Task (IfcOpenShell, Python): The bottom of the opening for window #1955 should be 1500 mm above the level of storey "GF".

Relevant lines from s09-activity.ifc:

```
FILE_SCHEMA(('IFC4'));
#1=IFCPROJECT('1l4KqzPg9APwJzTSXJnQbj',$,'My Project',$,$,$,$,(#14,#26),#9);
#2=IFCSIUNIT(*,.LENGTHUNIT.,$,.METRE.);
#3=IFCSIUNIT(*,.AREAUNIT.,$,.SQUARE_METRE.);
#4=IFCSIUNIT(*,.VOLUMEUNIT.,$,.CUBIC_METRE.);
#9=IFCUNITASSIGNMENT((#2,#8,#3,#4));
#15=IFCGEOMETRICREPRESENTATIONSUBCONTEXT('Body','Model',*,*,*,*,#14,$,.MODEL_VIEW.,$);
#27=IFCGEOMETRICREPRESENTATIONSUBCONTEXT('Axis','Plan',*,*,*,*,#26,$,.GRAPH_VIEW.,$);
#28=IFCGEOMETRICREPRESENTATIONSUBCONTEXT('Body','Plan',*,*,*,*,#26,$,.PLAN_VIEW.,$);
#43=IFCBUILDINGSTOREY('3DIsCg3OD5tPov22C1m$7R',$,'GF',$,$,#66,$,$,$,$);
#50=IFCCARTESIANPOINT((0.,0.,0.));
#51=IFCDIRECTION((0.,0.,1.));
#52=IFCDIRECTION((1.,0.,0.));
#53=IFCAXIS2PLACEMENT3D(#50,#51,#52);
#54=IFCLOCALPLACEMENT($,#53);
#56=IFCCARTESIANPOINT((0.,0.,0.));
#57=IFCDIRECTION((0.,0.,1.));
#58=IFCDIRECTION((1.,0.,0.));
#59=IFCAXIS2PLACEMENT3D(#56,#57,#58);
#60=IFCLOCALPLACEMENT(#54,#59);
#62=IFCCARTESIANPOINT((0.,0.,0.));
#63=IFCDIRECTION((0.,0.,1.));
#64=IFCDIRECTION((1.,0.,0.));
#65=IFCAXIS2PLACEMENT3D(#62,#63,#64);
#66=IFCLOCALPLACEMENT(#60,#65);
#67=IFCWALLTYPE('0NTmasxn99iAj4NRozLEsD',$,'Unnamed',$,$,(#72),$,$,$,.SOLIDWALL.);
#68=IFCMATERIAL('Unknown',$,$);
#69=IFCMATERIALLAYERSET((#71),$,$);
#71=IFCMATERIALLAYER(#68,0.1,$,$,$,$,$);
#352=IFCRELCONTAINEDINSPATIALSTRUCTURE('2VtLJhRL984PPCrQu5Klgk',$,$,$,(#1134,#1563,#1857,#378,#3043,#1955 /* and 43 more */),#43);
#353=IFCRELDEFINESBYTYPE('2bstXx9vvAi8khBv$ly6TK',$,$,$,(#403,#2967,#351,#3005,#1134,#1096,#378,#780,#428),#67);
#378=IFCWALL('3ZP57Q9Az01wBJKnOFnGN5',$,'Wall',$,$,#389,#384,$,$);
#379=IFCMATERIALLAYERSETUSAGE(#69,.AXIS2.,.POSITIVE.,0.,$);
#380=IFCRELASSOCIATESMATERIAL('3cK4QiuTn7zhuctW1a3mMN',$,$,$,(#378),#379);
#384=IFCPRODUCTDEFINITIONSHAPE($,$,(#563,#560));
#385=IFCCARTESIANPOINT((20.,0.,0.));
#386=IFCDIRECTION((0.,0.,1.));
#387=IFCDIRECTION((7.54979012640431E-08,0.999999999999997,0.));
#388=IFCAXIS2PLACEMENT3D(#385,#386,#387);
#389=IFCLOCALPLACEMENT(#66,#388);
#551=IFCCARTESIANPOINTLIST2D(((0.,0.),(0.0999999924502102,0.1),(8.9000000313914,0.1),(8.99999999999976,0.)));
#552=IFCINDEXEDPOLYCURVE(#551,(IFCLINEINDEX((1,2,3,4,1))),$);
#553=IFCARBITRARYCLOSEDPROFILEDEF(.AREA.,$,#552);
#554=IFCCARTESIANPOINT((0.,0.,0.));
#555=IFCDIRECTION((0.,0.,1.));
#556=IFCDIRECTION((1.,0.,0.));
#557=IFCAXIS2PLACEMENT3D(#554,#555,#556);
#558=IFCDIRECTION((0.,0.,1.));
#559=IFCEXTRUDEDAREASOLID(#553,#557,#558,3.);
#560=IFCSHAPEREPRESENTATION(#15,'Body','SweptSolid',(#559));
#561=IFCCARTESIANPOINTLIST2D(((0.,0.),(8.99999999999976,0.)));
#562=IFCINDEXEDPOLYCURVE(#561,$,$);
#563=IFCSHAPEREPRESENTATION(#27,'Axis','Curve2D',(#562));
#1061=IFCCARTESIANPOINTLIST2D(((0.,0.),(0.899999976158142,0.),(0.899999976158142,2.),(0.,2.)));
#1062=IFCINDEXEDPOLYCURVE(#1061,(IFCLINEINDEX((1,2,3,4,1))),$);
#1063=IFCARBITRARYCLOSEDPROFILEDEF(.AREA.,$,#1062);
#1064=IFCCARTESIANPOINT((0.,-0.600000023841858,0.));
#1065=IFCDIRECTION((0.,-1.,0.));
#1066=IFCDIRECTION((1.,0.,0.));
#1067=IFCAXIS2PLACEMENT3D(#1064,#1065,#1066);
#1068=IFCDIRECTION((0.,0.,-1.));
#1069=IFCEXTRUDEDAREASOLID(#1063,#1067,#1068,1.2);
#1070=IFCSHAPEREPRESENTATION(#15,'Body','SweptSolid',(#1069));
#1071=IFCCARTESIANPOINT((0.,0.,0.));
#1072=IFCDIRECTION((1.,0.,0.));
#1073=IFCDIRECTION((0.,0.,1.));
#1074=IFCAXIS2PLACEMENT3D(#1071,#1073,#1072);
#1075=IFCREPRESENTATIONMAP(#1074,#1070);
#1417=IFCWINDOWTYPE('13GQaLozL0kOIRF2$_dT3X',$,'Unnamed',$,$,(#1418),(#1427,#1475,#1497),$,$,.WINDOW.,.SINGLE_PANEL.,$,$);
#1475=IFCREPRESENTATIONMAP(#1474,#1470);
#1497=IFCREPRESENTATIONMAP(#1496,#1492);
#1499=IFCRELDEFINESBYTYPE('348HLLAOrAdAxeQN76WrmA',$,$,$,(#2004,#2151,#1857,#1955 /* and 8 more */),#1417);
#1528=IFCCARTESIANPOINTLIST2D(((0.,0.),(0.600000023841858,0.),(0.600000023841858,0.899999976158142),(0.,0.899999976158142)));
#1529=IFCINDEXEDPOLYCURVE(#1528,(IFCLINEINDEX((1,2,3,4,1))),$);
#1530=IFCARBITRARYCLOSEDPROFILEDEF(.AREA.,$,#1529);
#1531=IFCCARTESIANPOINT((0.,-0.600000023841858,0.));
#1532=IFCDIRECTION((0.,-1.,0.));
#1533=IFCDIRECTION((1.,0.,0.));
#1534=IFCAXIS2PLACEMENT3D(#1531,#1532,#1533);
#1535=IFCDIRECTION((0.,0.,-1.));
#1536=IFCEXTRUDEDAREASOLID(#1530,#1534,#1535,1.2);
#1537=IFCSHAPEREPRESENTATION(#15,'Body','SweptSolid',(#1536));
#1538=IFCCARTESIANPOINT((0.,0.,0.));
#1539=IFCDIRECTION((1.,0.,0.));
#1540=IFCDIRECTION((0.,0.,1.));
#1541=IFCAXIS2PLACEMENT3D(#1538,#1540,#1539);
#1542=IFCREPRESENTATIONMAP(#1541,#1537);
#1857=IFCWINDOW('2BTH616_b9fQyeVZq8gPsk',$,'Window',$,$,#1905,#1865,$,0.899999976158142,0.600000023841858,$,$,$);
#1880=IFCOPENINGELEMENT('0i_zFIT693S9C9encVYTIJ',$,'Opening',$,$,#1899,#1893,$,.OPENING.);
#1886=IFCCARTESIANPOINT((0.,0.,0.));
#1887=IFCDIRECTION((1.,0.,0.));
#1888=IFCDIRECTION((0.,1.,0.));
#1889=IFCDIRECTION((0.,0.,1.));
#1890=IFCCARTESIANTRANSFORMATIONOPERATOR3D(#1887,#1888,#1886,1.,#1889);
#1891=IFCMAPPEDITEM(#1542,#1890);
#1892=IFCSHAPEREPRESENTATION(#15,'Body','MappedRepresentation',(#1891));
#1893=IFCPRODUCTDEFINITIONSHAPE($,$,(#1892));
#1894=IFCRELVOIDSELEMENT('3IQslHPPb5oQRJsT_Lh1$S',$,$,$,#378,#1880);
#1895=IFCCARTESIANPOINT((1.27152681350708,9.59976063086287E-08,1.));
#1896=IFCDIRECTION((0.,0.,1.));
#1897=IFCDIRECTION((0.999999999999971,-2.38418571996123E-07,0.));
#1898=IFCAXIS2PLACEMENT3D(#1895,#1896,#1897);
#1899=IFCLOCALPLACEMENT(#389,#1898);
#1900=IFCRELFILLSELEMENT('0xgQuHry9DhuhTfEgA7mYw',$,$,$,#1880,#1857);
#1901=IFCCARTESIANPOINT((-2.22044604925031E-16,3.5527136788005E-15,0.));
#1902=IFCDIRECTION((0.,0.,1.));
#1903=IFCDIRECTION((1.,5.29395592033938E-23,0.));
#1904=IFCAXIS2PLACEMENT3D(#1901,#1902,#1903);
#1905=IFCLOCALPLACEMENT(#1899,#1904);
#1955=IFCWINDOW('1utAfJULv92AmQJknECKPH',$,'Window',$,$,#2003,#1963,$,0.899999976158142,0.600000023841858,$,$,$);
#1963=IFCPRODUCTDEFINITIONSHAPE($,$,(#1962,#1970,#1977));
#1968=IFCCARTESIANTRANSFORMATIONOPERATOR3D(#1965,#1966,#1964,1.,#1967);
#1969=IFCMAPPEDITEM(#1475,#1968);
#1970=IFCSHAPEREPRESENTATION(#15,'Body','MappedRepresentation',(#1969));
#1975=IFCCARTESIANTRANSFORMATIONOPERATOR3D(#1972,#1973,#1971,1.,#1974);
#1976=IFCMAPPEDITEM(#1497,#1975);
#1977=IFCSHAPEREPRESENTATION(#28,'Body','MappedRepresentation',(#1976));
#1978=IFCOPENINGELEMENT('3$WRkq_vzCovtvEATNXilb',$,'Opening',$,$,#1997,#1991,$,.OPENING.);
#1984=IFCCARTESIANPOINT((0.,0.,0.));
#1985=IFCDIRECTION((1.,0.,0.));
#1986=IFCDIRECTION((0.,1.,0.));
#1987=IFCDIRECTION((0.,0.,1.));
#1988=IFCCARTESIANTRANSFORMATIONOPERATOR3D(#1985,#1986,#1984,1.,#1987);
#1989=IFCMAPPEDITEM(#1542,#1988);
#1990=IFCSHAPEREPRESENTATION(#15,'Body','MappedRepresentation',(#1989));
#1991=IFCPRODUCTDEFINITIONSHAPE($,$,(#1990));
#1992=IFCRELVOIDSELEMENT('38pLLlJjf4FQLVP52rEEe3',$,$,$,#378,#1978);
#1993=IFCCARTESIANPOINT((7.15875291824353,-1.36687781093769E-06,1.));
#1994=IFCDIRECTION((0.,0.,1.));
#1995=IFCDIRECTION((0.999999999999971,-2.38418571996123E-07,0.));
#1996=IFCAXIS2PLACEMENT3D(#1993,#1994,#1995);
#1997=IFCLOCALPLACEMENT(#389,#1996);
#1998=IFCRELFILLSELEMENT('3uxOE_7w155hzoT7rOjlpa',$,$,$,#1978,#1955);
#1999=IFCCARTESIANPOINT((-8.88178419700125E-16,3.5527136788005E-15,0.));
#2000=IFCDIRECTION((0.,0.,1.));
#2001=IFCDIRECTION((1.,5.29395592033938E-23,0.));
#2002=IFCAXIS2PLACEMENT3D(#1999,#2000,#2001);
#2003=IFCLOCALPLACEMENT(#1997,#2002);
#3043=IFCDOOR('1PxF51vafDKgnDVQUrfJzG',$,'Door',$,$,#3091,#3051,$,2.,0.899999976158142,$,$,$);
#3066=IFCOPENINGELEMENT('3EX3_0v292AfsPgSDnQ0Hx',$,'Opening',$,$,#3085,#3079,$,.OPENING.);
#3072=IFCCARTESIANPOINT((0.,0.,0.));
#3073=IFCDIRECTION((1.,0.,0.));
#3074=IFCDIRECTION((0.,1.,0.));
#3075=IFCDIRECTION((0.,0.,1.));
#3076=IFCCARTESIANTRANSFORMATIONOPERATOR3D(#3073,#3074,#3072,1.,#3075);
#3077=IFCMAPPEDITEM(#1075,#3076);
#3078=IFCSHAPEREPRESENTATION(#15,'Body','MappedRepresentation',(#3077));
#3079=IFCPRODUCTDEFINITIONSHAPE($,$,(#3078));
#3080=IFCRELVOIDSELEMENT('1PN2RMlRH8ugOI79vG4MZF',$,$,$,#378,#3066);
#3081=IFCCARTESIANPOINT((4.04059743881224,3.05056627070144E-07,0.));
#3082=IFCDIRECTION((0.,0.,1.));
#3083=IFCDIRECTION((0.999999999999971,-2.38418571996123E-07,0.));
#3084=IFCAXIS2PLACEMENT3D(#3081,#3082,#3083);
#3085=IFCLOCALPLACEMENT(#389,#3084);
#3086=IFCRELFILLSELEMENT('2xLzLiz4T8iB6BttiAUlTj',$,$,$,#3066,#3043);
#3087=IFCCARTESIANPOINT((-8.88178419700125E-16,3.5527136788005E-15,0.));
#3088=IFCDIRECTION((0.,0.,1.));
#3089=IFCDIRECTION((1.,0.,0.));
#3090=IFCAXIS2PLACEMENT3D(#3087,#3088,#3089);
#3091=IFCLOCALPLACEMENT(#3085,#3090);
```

```python
import numpy as np
import ifcopenshell
import ifcopenshell.api.geometry
import ifcopenshell.geom
import ifcopenshell.util.element
import ifcopenshell.util.placement
import ifcopenshell.util.shape
import ifcopenshell.util.unit

model = ifcopenshell.open("s09-activity.ifc")
unit_scale = ifcopenshell.util.unit.calculate_unit_scale(model)

window = model.by_guid("1utAfJULv92AmQJknECKPH")
opening = window.FillsVoids[0].RelatingOpeningElement
storey = ifcopenshell.util.element.get_container(window, ifc_class="IfcBuildingStorey")
level = ifcopenshell.util.placement.get_local_placement(storey.ObjectPlacement)[2, 3]

# The opening's origin need not be at the sill, so measure its lowest point.
shape = ifcopenshell.geom.create_shape(ifcopenshell.geom.settings(), opening)
bottom = ifcopenshell.util.shape.get_shape_bottom_elevation(shape, shape.geometry) / unit_scale
dz = level + 1.5 / unit_scale - bottom

shift = np.array([0.0, 0.0, dz])
# The window is placed relative to its opening, so it follows when the opening moves.
matrix = ifcopenshell.util.placement.get_local_placement(opening.ObjectPlacement)
matrix[:3, 3] += shift
ifcopenshell.api.geometry.edit_object_placement(
    model, product=opening, matrix=matrix, is_si=False, should_transform_children=True
)

print(f"moved by {dz * unit_scale:+.3f} m")

model.write("s09-activity_rev.ifc")
```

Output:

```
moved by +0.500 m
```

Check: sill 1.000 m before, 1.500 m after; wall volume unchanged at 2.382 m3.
